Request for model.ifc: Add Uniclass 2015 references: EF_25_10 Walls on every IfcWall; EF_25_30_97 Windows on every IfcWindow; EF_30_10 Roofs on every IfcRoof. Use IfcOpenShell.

First a look at what the model holds.

```python
import ifcopenshell

model = ifcopenshell.open("model.ifc")
print(model.schema)
print("classifications:", [c.Name for c in model.by_type("IfcClassification")])
for ifc_class in ("IfcDoor", "IfcRoof", "IfcStair", "IfcWall", "IfcWindow"):
    print(ifc_class, len(model.by_type(ifc_class)))
```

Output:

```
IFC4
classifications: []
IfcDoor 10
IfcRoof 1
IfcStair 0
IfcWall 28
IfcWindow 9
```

```python
import ifcopenshell
import ifcopenshell.api.classification

model = ifcopenshell.open("model.ifc")

system = ifcopenshell.api.classification.add_classification(model, classification="Uniclass 2015")

codes = {
    "IfcWall": ("EF_25_10", "Walls"),
    "IfcWindow": ("EF_25_30_97", "Windows"),
    "IfcRoof": ("EF_30_10", "Roofs"),
}
for ifc_class, (code, name) in codes.items():
    products = model.by_type(ifc_class)
    ifcopenshell.api.classification.add_reference(
        model, products=products, classification=system, identification=code, name=name
    )
    print(code, len(products))

model.write("model_v2.ifc")
```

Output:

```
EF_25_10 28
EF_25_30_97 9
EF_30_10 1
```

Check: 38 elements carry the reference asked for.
